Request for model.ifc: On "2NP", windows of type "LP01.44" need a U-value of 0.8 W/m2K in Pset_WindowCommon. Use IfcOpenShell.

First a look at what the model holds.

```python
import ifcopenshell
import ifcopenshell.util.element

model = ifcopenshell.open("model.ifc")
print(model.schema)
storey = next(s for s in model.by_type("IfcBuildingStorey") if s.Name == "2NP")
windows = [e for e in ifcopenshell.util.element.get_decomposition(storey) if e.is_a("IfcWindow")]
seen = {}
for e in windows:
    element_type = ifcopenshell.util.element.get_type(e)
    key = (element_type.Name if element_type != e and element_type else None, ifcopenshell.util.element.get_pset(e, "Pset_WindowCommon", "ThermalTransmittance"))
    seen[key] = seen.get(key, 0) + 1
for (name, value), count in sorted(seen.items(), key=str):
    print(count, "x", name, "|", value)
```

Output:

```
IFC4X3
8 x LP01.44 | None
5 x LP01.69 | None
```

```python
import ifcopenshell
import ifcopenshell.api.pset
import ifcopenshell.util.element

model = ifcopenshell.open("model.ifc")

storey = next(s for s in model.by_type("IfcBuildingStorey") if s.Name == "2NP")
windows = [e for e in ifcopenshell.util.element.get_decomposition(storey) if e.is_a("IfcWindow")]

count = 0
for e in windows:
    element_type = ifcopenshell.util.element.get_type(e)
    if element_type in (None, e) or element_type.Name != "LP01.44":
        continue
    # add_pset returns the element's existing set when there is one.
    pset = ifcopenshell.api.pset.add_pset(model, product=e, name="Pset_WindowCommon")
    ifcopenshell.api.pset.edit_pset(model, pset=pset, properties={"ThermalTransmittance": 0.8})
    count += 1

print(count, "windows updated")

model.write("model-out.ifc")
```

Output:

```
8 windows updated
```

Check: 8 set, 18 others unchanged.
